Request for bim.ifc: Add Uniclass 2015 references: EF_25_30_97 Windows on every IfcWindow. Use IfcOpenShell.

First a look at what the model holds.

```python
import ifcopenshell

model = ifcopenshell.open("bim.ifc")
print(model.schema)
print("classifications:", [c.Name for c in model.by_type("IfcClassification")])
for ifc_class in ("IfcDoor", "IfcRoof", "IfcStair", "IfcWall", "IfcWindow"):
    print(ifc_class, len(model.by_type(ifc_class)))
```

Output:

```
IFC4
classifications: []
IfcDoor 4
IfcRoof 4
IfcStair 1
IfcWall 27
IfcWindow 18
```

```python
import ifcopenshell
import ifcopenshell.api.classification

model = ifcopenshell.open("bim.ifc")

system = ifcopenshell.api.classification.add_classification(model, classification="Uniclass 2015")

codes = {
    "IfcWindow": ("EF_25_30_97", "Windows"),
}
for ifc_class, (code, name) in codes.items():
    products = model.by_type(ifc_class)
    ifcopenshell.api.classification.add_reference(
        model, products=products, classification=system, identification=code, name=name
    )
    print(code, len(products))

model.write("bim_updated.ifc")
```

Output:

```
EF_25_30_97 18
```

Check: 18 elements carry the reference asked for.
